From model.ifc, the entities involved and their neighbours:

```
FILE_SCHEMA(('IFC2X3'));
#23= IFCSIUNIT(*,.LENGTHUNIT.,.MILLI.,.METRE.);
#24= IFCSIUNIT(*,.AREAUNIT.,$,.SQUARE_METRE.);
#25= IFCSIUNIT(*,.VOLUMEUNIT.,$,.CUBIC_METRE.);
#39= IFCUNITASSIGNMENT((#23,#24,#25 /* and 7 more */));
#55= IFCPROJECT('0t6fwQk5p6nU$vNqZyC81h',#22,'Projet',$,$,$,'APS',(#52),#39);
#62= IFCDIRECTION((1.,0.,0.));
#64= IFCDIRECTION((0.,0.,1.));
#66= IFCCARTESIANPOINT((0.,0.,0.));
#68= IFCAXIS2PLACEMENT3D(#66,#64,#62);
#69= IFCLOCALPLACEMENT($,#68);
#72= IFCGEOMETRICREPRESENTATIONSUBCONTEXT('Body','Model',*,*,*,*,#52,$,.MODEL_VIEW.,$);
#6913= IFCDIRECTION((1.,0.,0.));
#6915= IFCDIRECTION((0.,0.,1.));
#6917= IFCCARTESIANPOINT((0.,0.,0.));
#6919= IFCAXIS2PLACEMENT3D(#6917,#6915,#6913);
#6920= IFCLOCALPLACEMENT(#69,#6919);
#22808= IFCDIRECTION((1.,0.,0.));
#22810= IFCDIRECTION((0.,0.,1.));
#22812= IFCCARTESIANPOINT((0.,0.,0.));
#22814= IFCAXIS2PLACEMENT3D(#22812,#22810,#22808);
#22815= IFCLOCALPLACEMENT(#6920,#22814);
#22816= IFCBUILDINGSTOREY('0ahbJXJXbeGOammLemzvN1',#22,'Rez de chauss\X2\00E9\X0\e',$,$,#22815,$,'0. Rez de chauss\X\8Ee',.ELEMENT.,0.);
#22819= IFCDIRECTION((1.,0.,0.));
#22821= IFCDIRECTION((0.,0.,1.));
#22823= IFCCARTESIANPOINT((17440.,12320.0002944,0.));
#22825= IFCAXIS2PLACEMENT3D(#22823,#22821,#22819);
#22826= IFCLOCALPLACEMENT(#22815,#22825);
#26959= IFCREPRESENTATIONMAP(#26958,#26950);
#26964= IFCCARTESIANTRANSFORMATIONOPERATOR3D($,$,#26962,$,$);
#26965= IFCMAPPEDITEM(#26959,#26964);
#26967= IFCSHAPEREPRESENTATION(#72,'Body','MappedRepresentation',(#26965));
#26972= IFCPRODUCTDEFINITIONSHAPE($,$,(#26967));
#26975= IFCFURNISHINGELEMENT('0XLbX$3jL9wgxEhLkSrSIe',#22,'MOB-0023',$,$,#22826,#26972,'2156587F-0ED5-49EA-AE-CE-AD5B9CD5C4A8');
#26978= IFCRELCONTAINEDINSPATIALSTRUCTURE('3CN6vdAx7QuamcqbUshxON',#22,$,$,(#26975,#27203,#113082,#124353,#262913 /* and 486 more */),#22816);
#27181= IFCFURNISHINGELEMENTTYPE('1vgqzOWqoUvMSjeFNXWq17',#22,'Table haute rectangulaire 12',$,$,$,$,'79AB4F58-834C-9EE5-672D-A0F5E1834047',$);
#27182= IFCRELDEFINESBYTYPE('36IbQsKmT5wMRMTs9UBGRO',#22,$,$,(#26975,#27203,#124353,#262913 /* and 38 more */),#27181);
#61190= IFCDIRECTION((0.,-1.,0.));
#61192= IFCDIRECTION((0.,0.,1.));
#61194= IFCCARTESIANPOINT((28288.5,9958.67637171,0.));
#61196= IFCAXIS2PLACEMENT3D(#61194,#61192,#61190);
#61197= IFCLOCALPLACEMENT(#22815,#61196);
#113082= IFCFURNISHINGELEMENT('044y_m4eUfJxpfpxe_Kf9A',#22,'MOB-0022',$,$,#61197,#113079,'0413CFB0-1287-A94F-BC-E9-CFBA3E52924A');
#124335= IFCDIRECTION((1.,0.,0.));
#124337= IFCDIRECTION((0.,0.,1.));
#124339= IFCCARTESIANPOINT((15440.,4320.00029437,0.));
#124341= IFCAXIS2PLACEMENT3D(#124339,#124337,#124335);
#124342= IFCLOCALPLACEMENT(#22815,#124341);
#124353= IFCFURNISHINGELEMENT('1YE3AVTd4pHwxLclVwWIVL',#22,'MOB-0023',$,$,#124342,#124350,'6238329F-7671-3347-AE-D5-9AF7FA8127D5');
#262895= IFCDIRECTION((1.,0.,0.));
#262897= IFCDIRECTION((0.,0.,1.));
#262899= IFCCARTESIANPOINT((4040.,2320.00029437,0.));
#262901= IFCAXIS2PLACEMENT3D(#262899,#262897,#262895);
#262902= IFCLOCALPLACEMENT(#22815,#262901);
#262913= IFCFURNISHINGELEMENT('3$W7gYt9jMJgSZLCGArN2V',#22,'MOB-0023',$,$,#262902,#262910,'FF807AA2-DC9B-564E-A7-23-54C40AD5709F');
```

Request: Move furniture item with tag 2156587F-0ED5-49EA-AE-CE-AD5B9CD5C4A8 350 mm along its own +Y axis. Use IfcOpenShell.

```python
import ifcopenshell
import ifcopenshell.api.geometry
import ifcopenshell.util.placement

model = ifcopenshell.open("model.ifc")

item = model.by_id(26975)
matrix = ifcopenshell.util.placement.get_local_placement(item.ObjectPlacement)
matrix[:3, 3] += matrix[:3, 1] * 350.0
ifcopenshell.api.geometry.edit_object_placement(model, product=item, matrix=matrix, is_si=False)

print(ifcopenshell.util.placement.get_local_placement(item.ObjectPlacement).round(3) + 0.0)

model.write("model_v2.ifc")
```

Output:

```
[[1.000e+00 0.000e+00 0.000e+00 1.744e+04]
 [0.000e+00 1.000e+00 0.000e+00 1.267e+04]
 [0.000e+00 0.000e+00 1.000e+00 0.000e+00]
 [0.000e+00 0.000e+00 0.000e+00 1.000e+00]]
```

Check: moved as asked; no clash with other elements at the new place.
